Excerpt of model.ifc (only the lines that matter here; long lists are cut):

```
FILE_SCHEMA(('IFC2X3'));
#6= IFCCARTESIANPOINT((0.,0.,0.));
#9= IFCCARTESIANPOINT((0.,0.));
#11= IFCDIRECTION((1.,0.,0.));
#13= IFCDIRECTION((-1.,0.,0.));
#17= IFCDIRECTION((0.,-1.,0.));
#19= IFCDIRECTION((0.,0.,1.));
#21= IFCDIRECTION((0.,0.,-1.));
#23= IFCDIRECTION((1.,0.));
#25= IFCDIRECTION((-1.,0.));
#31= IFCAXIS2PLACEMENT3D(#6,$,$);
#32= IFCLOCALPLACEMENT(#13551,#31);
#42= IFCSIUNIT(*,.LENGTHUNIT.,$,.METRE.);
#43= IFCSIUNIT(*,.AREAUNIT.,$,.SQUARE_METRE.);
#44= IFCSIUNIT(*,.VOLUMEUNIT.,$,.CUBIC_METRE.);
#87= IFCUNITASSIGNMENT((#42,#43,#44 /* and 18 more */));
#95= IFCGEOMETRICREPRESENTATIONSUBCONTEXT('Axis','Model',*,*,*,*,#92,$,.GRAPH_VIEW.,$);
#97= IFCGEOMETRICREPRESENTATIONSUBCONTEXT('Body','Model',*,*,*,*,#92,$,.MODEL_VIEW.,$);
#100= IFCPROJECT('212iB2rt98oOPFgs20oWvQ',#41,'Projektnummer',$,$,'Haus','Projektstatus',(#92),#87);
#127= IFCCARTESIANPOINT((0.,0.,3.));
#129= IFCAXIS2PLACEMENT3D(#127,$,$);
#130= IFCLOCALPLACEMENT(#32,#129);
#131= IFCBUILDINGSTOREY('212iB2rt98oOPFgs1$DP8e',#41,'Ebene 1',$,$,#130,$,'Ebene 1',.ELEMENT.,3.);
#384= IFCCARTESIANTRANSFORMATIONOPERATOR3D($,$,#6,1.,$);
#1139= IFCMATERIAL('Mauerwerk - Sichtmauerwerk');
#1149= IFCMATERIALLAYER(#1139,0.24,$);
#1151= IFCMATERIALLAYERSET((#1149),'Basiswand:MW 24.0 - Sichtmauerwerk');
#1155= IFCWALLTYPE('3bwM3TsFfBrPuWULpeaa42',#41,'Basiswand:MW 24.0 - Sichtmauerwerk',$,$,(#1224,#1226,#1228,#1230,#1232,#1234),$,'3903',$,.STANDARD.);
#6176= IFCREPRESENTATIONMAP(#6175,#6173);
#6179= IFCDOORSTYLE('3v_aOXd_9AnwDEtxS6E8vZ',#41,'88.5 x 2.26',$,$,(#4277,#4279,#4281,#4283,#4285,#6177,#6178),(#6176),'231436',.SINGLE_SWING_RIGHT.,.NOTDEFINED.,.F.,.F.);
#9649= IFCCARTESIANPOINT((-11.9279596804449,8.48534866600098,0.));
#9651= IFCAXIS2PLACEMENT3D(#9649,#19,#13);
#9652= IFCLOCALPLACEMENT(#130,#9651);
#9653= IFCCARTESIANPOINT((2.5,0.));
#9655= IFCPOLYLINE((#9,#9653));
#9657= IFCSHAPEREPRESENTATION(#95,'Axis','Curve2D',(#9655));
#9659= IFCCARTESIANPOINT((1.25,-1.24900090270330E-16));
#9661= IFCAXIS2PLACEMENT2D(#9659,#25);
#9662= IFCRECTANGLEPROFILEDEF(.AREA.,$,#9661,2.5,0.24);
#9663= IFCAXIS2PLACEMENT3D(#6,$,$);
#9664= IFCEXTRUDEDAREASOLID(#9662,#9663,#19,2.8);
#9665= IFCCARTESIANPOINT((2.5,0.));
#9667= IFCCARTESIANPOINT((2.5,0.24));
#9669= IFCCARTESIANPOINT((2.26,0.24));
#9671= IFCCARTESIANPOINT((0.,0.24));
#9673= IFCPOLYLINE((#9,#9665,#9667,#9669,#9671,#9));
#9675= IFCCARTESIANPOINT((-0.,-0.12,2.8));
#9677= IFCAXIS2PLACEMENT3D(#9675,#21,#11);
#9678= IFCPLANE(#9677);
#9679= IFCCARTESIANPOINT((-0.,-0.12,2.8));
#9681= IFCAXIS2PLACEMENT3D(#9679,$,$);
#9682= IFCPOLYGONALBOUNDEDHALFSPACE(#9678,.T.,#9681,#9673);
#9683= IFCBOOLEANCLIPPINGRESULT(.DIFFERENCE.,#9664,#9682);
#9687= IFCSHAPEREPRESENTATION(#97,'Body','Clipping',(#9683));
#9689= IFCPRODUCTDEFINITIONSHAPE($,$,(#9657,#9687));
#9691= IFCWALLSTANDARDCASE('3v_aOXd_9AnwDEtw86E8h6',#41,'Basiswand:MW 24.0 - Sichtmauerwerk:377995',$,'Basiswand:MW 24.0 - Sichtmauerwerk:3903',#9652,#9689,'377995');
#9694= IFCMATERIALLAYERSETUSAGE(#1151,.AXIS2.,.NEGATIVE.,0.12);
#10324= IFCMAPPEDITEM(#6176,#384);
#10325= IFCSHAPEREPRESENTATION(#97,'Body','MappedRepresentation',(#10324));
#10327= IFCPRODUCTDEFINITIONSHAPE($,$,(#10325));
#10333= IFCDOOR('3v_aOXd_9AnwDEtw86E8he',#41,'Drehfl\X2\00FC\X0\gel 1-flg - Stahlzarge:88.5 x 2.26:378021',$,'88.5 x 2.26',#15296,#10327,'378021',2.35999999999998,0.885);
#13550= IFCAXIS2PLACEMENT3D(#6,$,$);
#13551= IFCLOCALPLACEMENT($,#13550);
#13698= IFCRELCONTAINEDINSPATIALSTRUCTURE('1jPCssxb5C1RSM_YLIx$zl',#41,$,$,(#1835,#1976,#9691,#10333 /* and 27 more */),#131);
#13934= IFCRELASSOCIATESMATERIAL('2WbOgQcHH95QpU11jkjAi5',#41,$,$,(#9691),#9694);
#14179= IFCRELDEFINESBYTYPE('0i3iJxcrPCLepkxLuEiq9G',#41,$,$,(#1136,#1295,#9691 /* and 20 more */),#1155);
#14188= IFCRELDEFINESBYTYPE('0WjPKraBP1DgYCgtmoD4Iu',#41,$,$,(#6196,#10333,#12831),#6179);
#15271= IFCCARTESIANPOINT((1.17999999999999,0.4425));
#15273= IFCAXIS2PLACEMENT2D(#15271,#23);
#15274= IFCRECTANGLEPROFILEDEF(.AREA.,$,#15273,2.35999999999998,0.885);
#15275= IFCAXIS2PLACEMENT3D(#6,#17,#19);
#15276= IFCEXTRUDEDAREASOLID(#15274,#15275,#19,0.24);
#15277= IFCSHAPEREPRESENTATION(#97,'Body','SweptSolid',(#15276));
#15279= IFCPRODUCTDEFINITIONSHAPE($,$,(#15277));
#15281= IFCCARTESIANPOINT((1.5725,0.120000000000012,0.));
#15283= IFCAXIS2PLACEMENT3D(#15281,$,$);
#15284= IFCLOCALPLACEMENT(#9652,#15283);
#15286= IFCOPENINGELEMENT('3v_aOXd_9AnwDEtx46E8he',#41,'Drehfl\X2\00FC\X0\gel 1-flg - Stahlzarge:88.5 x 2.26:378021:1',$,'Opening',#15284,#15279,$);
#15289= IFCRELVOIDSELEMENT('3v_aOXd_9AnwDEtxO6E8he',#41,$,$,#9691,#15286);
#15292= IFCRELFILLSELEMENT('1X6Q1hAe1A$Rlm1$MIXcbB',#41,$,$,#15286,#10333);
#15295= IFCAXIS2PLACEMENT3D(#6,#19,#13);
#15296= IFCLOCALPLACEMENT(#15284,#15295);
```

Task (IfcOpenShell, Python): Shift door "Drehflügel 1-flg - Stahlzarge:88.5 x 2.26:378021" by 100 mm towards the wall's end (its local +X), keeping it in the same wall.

```python
import ifcopenshell
import ifcopenshell.api.geometry
import ifcopenshell.util.placement

model = ifcopenshell.open("model.ifc")

door = model.by_guid("3v_aOXd_9AnwDEtw86E8he")
opening = door.FillsVoids[0].RelatingOpeningElement
wall = opening.VoidsElements[0].RelatingBuildingElement

wall_matrix = ifcopenshell.util.placement.get_local_placement(wall.ObjectPlacement)
shift = wall_matrix[:3, 0] * 0.1
before = ifcopenshell.util.placement.get_local_placement(door.ObjectPlacement)[:3, 3].copy()

# The door is placed relative to its opening, so it follows when the opening moves.
matrix = ifcopenshell.util.placement.get_local_placement(opening.ObjectPlacement)
matrix[:3, 3] += shift
ifcopenshell.api.geometry.edit_object_placement(
    model, product=opening, matrix=matrix, is_si=False, should_transform_children=True
)

after = ifcopenshell.util.placement.get_local_placement(door.ObjectPlacement)[:3, 3]
print("door moved by", (after - before).round(3) + 0.0)

model.write("model-out.ifc")
```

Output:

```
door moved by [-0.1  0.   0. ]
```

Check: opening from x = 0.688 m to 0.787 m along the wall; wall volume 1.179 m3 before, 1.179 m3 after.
